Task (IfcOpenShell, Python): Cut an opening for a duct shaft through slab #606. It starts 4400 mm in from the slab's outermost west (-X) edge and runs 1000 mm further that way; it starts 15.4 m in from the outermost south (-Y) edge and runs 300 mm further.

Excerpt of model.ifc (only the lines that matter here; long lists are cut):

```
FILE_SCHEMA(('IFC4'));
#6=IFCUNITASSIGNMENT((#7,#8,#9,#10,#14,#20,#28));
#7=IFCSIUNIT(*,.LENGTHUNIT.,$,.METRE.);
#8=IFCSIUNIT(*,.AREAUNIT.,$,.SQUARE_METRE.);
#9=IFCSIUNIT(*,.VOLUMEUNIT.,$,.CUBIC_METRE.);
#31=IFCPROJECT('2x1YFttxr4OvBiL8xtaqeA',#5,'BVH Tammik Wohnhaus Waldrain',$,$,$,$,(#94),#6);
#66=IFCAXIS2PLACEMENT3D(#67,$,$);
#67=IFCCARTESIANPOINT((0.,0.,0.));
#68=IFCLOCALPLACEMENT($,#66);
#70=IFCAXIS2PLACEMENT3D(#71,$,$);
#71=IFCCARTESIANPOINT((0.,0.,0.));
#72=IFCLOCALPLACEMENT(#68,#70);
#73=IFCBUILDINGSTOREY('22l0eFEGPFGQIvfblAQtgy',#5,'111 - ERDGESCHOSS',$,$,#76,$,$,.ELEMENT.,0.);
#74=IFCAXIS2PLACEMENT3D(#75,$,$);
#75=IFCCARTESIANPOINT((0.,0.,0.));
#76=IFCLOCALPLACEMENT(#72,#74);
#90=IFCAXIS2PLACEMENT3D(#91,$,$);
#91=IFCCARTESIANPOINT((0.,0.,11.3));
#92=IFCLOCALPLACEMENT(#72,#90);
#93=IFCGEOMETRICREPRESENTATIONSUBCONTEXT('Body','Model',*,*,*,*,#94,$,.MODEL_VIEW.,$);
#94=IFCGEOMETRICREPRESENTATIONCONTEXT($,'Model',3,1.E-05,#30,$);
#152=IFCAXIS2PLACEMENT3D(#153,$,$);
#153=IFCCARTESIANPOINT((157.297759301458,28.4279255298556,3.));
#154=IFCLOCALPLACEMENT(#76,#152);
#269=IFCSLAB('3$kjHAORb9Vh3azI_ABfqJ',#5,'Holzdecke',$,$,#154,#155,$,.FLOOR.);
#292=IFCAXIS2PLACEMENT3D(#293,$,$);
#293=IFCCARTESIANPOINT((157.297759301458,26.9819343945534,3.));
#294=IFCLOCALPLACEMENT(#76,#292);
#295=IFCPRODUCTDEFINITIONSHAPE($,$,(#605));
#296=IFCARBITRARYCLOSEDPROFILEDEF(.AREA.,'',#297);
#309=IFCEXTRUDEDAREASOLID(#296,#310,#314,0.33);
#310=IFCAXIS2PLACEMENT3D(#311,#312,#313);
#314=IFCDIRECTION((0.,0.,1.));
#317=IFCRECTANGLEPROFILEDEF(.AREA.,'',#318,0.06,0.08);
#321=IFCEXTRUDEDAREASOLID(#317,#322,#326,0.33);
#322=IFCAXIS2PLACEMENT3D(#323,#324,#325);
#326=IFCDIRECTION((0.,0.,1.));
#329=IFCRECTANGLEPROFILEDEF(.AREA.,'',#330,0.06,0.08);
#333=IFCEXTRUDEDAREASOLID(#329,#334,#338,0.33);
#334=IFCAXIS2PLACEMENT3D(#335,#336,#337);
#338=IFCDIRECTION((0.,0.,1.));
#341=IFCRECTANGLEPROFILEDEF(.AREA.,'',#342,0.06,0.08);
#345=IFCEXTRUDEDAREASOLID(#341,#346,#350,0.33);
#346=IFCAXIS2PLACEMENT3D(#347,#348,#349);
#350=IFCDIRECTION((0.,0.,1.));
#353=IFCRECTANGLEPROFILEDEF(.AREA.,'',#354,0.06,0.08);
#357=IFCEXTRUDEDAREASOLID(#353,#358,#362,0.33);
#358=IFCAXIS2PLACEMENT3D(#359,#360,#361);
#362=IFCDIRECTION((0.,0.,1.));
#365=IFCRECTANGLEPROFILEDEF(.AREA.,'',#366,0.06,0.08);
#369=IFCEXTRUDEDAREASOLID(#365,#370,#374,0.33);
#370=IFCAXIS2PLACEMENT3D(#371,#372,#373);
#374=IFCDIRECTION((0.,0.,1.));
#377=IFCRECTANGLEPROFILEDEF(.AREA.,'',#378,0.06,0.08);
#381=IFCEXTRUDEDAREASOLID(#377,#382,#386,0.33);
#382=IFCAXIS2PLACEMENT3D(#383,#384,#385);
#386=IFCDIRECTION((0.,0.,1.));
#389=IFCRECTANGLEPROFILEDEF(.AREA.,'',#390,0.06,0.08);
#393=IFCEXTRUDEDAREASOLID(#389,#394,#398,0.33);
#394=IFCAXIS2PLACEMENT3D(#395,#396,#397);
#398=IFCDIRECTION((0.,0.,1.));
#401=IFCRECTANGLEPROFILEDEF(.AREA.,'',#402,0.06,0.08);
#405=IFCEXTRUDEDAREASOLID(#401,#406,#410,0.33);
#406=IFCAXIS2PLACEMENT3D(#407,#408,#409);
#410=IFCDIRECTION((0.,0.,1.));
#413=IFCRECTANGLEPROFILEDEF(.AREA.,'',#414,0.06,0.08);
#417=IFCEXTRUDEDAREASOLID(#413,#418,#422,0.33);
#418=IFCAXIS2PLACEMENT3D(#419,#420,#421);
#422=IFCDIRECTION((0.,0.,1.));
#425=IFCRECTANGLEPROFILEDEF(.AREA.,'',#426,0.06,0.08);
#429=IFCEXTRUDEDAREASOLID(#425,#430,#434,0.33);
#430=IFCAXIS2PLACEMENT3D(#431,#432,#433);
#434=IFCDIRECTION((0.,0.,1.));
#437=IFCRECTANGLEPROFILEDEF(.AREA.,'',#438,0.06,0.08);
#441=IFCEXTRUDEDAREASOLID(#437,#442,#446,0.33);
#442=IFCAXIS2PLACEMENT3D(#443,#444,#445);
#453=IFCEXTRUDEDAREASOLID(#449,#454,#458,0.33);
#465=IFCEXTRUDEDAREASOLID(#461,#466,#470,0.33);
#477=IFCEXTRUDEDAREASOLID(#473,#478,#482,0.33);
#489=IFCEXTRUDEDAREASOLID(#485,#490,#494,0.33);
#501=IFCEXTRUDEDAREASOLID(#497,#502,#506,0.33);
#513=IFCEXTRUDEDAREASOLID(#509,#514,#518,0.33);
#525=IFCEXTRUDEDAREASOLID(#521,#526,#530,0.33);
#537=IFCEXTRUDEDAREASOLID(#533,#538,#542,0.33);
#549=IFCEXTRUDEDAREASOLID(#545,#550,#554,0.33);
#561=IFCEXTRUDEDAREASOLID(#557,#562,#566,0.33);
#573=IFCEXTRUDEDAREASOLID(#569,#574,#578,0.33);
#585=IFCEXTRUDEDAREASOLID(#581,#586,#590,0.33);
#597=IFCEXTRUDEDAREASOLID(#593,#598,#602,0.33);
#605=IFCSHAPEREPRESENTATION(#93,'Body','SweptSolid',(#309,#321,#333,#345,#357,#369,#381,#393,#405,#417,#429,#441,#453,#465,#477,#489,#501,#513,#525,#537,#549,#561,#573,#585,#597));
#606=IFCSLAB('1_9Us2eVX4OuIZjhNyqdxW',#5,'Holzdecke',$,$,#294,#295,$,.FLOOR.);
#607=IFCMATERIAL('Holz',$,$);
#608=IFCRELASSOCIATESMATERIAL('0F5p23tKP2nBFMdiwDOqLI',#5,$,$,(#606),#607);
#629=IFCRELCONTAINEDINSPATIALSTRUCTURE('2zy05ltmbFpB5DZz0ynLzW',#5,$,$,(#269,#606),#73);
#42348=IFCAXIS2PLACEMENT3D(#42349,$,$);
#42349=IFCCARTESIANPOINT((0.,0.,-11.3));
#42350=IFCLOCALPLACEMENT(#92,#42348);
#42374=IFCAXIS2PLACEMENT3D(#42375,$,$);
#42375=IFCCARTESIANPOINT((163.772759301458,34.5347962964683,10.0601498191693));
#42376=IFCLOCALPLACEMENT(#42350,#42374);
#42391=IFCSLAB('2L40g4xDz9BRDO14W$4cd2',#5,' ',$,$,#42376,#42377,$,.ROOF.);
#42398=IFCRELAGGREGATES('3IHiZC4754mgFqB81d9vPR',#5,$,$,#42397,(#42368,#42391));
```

```python
import numpy as np
import ifcopenshell
import ifcopenshell.api.feature
import ifcopenshell.api.geometry
import ifcopenshell.api.root
import ifcopenshell.geom
import ifcopenshell.util.placement
import ifcopenshell.util.representation
import ifcopenshell.util.shape
import ifcopenshell.util.unit

model = ifcopenshell.open("model.ifc")
unit_scale = ifcopenshell.util.unit.calculate_unit_scale(model)
settings = ifcopenshell.geom.settings()


def volume(element):
    """Net volume in cubic metres, openings subtracted."""
    shape = ifcopenshell.geom.create_shape(settings, element)
    return ifcopenshell.util.shape.get_volume(shape.geometry)


slab = model.by_guid("1_9Us2eVX4OuIZjhNyqdxW")
before = volume(slab)

# Extent in the slab's own axes, in metres. The edges named are its -X and -Y sides.
slab_shape = ifcopenshell.geom.create_shape(settings, slab)
vertices = ifcopenshell.util.shape.get_vertices(slab_shape.geometry)
x_min, y_min, bottom = vertices.min(axis=0)
top = vertices[:, 2].max()

opening = ifcopenshell.api.root.create_entity(model, ifc_class="IfcOpeningElement", name="Duct shaft opening", predefined_type="OPENING")
context = ifcopenshell.util.representation.get_context(model, "Model", "Body", "MODEL_VIEW")
width, depth = 1, 0.3
outline = [(0.0, 0.0), (width, 0.0), (width, depth), (0.0, depth), (0.0, 0.0)]
# Overshoot both faces by 50 mm so the cut is clean.
shape = ifcopenshell.api.geometry.add_slab_representation(
    model, context=context, depth=top - bottom + 0.1, polyline=outline
)
ifcopenshell.api.geometry.assign_representation(model, product=opening, representation=shape)

matrix = ifcopenshell.util.placement.get_local_placement(slab.ObjectPlacement)
matrix[:, 3] = matrix @ np.append(np.array([x_min + 4.4, y_min + 15.4, bottom - 0.05]) / unit_scale, 1.0)
ifcopenshell.api.geometry.edit_object_placement(model, product=opening, matrix=matrix, is_si=False)
ifcopenshell.api.feature.add_feature(model, feature=opening, element=slab)

after = volume(slab)

print(f"slab volume {before:.3f} -> {after:.3f} m3")

model.write("model_rev.ifc")
```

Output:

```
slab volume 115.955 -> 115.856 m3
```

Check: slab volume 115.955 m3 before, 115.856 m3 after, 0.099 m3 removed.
